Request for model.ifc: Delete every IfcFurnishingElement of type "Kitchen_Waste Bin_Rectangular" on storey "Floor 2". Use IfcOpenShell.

First a look at what the model holds.

```python
import ifcopenshell
import ifcopenshell.util.element

model = ifcopenshell.open("model.ifc")
print(model.schema)
storey = next(s for s in model.by_type("IfcBuildingStorey") if s.Name == "Floor 2")
furniture = [e for e in ifcopenshell.util.element.get_decomposition(storey) if e.is_a("IfcFurnishingElement")]
seen = {}
for e in furniture:
    element_type = ifcopenshell.util.element.get_type(e)
    name = element_type.Name if element_type not in (None, e) else None
    seen[name] = seen.get(name, 0) + 1
for name, count in sorted(seen.items(), key=str):
    print(count, "x", name)
```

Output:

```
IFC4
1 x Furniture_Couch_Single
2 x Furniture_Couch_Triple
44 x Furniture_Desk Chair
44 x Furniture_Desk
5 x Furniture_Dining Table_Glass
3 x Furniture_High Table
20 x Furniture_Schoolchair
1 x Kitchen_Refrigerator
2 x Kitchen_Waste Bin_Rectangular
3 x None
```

```python
import ifcopenshell
import ifcopenshell.api.root
import ifcopenshell.util.element

model = ifcopenshell.open("model.ifc")

storey = next(s for s in model.by_type("IfcBuildingStorey") if s.Name == "Floor 2")
furniture = [e for e in ifcopenshell.util.element.get_decomposition(storey) if e.is_a("IfcFurnishingElement")]
targets = [e for e in furniture if (t := ifcopenshell.util.element.get_type(e)) not in (None, e) and t.Name == "Kitchen_Waste Bin_Rectangular"]

for e in targets:
    ifcopenshell.api.root.remove_product(model, product=e)
print(len(targets), "removed")

model.write("model_rev.ifc")
```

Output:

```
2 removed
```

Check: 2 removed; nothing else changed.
